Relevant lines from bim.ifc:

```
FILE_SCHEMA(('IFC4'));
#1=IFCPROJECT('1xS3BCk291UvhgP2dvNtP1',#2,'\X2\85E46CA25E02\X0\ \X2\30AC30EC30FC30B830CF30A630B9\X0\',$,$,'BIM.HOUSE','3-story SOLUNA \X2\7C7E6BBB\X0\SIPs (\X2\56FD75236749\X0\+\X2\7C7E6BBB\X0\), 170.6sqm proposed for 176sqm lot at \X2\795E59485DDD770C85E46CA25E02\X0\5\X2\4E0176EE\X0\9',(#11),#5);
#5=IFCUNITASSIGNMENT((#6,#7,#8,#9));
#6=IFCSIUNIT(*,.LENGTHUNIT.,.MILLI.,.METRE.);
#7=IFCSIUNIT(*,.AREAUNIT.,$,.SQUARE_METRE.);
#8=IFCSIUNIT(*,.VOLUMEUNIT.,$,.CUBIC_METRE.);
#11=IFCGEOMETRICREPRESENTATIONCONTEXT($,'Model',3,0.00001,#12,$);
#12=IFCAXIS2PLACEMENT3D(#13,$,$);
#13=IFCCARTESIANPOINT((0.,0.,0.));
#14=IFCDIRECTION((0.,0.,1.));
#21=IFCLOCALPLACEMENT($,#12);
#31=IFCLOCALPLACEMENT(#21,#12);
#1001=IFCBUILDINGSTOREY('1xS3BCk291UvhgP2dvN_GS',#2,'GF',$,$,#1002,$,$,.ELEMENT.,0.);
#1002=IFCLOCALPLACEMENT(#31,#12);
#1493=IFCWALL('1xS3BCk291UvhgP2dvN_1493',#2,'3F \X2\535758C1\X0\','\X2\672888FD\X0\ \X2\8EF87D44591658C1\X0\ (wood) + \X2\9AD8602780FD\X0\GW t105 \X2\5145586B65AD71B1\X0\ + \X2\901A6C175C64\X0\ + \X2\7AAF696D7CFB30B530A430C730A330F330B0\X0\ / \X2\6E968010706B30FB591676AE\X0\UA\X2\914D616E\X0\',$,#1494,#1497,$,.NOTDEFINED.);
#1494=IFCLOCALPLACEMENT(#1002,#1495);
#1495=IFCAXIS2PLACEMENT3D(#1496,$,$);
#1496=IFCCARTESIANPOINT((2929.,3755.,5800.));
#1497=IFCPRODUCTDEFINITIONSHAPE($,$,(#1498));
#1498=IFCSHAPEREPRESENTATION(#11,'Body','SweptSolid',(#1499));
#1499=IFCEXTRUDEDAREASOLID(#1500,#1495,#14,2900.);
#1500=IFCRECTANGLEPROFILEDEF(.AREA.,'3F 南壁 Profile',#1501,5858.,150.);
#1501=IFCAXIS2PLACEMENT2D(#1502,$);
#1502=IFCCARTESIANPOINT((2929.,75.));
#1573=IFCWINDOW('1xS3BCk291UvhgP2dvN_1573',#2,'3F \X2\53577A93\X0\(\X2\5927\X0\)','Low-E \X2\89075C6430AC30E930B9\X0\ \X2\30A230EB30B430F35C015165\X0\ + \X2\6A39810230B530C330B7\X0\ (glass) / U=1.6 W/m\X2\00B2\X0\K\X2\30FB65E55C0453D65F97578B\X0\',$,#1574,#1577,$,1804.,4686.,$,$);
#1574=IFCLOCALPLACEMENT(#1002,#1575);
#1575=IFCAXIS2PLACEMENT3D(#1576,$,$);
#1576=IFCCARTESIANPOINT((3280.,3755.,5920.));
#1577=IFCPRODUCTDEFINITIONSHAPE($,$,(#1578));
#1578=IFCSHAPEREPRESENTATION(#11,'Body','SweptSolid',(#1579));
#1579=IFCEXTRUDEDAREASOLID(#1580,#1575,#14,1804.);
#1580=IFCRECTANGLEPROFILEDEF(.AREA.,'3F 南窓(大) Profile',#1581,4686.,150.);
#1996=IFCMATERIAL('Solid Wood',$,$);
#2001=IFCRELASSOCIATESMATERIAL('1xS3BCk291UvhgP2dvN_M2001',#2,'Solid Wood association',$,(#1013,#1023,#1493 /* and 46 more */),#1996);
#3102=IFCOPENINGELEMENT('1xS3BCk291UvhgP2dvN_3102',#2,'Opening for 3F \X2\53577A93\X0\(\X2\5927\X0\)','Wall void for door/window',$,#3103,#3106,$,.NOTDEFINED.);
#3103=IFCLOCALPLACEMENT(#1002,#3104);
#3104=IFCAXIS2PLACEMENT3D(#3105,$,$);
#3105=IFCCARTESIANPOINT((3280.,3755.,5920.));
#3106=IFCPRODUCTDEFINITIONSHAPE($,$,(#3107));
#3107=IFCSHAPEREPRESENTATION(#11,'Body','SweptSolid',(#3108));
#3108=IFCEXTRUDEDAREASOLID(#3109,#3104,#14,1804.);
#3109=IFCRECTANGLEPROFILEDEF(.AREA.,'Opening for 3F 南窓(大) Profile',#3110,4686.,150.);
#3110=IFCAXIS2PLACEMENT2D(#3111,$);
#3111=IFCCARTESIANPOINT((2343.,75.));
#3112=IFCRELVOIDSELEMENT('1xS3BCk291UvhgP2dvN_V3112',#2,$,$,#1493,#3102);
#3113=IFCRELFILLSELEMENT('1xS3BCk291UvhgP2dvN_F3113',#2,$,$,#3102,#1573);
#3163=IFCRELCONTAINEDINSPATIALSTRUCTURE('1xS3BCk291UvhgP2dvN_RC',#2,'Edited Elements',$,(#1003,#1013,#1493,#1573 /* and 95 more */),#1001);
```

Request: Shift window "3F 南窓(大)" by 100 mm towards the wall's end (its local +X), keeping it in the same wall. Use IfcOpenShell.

```python
import ifcopenshell
import ifcopenshell.api.geometry
import ifcopenshell.util.placement

model = ifcopenshell.open("bim.ifc")

window = model.by_guid("1xS3BCk291UvhgP2dvN_1573")
opening = window.FillsVoids[0].RelatingOpeningElement
wall = opening.VoidsElements[0].RelatingBuildingElement

wall_matrix = ifcopenshell.util.placement.get_local_placement(wall.ObjectPlacement)
shift = wall_matrix[:3, 0] * 100.0
before = ifcopenshell.util.placement.get_local_placement(window.ObjectPlacement)[:3, 3].copy()

# The window is not placed relative to its opening, so move both.
for product in (opening, window):
    matrix = ifcopenshell.util.placement.get_local_placement(product.ObjectPlacement)
    matrix[:3, 3] += shift
    ifcopenshell.api.geometry.edit_object_placement(model, product=product, matrix=matrix, is_si=False)

after = ifcopenshell.util.placement.get_local_placement(window.ObjectPlacement)[:3, 3]
print("window moved by", (after - before).round(3) + 0.0)

model.write("bim_updated.ifc")
```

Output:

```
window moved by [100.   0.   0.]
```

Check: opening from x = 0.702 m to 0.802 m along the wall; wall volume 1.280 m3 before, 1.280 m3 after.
